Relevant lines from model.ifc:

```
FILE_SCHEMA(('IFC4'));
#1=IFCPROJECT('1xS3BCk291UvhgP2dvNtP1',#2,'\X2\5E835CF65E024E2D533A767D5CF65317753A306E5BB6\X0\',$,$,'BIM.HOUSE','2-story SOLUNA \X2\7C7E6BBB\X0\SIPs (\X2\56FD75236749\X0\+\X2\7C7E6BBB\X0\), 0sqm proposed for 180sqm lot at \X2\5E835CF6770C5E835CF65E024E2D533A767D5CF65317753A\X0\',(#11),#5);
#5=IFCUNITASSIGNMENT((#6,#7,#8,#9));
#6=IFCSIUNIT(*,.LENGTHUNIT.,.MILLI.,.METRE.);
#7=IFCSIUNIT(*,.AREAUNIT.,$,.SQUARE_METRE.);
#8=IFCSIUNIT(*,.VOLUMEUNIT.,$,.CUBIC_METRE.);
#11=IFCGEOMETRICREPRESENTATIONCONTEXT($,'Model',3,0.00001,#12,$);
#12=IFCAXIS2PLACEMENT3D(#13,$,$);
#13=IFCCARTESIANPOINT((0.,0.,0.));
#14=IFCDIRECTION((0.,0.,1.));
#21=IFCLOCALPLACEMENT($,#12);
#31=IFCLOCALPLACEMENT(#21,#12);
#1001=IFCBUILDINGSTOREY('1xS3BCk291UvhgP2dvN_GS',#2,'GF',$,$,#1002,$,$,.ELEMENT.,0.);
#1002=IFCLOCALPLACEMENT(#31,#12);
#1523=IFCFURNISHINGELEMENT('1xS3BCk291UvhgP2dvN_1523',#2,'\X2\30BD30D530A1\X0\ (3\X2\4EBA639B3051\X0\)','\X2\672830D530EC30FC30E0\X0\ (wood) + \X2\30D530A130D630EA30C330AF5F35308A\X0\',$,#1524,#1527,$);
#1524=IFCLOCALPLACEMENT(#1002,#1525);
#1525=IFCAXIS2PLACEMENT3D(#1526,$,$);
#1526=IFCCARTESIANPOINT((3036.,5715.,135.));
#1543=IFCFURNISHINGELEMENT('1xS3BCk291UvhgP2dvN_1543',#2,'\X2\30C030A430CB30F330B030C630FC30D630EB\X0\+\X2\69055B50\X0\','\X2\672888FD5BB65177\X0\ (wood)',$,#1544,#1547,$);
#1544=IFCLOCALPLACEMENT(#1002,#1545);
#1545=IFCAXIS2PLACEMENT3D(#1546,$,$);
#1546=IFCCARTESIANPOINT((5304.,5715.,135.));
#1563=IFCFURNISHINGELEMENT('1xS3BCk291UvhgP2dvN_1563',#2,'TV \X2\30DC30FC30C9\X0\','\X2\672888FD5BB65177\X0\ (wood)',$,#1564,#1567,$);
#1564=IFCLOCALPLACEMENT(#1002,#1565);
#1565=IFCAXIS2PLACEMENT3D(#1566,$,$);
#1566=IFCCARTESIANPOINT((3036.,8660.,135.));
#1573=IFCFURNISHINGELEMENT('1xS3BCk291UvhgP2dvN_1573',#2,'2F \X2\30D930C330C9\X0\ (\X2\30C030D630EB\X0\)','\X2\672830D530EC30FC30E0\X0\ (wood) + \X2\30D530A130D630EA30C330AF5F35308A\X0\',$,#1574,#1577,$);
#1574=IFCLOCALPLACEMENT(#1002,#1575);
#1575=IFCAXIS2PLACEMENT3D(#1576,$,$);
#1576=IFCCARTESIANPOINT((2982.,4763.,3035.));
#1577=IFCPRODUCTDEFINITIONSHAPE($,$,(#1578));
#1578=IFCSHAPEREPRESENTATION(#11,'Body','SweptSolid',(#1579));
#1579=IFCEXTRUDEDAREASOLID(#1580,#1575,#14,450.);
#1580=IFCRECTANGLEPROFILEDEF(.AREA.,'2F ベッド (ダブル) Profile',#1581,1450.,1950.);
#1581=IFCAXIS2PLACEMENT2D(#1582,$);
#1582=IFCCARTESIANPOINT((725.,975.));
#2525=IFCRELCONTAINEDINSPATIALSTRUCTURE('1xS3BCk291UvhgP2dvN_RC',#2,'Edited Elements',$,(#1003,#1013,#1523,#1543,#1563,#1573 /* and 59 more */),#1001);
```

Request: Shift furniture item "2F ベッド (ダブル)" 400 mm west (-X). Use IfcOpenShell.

```python
import ifcopenshell
import ifcopenshell.api.geometry
import ifcopenshell.util.placement
import ifcopenshell.util.unit

model = ifcopenshell.open("model.ifc")
unit_scale = ifcopenshell.util.unit.calculate_unit_scale(model)

item = model.by_guid("1xS3BCk291UvhgP2dvN_1573")
matrix = ifcopenshell.util.placement.get_local_placement(item.ObjectPlacement)
matrix[0, 3] -= 0.4 / unit_scale
ifcopenshell.api.geometry.edit_object_placement(model, product=item, matrix=matrix, is_si=False)

print(ifcopenshell.util.placement.get_local_placement(item.ObjectPlacement).round(3) + 0.0)

model.write("model_updated.ifc")
```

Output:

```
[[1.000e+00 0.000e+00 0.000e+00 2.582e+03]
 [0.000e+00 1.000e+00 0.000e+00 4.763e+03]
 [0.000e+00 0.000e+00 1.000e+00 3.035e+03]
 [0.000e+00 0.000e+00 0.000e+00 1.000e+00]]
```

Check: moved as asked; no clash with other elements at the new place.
